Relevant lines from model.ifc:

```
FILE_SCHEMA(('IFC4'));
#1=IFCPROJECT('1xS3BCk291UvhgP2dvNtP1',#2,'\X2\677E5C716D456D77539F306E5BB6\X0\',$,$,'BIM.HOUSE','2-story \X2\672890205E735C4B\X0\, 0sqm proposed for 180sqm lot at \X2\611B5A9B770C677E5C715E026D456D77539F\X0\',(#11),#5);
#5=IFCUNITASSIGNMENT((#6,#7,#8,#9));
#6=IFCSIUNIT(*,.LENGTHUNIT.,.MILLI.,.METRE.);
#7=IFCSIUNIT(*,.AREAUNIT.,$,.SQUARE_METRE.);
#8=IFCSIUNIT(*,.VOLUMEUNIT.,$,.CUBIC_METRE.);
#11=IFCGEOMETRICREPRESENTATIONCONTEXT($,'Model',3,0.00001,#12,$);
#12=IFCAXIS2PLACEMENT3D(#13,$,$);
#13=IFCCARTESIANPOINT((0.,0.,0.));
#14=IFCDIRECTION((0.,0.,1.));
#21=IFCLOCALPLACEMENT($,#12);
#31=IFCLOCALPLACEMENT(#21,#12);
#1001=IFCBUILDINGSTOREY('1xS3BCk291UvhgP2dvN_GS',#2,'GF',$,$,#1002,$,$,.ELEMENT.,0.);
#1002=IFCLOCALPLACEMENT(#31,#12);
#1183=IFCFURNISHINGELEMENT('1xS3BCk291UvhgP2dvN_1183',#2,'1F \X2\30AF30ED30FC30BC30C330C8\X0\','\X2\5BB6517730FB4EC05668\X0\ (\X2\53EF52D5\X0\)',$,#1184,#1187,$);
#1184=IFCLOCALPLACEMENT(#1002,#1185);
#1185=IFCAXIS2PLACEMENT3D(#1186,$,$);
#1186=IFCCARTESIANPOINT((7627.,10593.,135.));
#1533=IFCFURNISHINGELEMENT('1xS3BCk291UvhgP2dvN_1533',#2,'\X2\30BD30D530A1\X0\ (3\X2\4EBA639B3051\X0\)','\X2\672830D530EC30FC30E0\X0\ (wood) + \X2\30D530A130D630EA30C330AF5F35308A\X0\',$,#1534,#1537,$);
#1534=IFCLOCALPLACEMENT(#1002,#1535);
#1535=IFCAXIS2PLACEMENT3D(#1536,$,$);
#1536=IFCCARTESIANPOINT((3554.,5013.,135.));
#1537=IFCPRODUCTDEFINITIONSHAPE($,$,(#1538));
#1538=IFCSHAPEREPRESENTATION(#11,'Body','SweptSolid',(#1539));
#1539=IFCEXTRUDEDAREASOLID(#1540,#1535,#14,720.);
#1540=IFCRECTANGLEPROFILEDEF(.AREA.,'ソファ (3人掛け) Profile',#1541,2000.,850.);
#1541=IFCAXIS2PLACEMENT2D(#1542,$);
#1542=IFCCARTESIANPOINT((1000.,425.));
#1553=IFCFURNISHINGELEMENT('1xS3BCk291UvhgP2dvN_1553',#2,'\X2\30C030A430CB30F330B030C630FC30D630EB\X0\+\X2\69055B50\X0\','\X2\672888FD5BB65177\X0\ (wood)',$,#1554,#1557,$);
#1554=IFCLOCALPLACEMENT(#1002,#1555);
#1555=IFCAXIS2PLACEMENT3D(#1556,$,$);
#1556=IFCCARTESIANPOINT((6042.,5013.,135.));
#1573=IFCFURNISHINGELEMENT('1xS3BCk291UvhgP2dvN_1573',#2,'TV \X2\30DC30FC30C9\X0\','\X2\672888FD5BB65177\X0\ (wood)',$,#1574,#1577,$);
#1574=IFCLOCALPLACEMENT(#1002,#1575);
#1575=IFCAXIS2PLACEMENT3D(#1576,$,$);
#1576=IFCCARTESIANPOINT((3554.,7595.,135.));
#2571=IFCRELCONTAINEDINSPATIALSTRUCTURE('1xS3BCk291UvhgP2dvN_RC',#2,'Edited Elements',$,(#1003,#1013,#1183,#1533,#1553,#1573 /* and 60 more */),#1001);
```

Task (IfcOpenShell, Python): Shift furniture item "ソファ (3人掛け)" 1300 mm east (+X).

```python
import ifcopenshell
import ifcopenshell.api.geometry
import ifcopenshell.util.placement
import ifcopenshell.util.unit

model = ifcopenshell.open("model.ifc")
unit_scale = ifcopenshell.util.unit.calculate_unit_scale(model)

item = model.by_id(1533)
matrix = ifcopenshell.util.placement.get_local_placement(item.ObjectPlacement)
matrix[0, 3] += 1.3 / unit_scale
ifcopenshell.api.geometry.edit_object_placement(model, product=item, matrix=matrix, is_si=False)

print(ifcopenshell.util.placement.get_local_placement(item.ObjectPlacement).round(3) + 0.0)

model.write("model_rev.ifc")
```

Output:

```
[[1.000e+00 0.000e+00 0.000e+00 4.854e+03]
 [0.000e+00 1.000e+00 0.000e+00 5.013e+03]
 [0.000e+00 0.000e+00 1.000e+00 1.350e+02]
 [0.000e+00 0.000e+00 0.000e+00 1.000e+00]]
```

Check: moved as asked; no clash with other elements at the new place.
